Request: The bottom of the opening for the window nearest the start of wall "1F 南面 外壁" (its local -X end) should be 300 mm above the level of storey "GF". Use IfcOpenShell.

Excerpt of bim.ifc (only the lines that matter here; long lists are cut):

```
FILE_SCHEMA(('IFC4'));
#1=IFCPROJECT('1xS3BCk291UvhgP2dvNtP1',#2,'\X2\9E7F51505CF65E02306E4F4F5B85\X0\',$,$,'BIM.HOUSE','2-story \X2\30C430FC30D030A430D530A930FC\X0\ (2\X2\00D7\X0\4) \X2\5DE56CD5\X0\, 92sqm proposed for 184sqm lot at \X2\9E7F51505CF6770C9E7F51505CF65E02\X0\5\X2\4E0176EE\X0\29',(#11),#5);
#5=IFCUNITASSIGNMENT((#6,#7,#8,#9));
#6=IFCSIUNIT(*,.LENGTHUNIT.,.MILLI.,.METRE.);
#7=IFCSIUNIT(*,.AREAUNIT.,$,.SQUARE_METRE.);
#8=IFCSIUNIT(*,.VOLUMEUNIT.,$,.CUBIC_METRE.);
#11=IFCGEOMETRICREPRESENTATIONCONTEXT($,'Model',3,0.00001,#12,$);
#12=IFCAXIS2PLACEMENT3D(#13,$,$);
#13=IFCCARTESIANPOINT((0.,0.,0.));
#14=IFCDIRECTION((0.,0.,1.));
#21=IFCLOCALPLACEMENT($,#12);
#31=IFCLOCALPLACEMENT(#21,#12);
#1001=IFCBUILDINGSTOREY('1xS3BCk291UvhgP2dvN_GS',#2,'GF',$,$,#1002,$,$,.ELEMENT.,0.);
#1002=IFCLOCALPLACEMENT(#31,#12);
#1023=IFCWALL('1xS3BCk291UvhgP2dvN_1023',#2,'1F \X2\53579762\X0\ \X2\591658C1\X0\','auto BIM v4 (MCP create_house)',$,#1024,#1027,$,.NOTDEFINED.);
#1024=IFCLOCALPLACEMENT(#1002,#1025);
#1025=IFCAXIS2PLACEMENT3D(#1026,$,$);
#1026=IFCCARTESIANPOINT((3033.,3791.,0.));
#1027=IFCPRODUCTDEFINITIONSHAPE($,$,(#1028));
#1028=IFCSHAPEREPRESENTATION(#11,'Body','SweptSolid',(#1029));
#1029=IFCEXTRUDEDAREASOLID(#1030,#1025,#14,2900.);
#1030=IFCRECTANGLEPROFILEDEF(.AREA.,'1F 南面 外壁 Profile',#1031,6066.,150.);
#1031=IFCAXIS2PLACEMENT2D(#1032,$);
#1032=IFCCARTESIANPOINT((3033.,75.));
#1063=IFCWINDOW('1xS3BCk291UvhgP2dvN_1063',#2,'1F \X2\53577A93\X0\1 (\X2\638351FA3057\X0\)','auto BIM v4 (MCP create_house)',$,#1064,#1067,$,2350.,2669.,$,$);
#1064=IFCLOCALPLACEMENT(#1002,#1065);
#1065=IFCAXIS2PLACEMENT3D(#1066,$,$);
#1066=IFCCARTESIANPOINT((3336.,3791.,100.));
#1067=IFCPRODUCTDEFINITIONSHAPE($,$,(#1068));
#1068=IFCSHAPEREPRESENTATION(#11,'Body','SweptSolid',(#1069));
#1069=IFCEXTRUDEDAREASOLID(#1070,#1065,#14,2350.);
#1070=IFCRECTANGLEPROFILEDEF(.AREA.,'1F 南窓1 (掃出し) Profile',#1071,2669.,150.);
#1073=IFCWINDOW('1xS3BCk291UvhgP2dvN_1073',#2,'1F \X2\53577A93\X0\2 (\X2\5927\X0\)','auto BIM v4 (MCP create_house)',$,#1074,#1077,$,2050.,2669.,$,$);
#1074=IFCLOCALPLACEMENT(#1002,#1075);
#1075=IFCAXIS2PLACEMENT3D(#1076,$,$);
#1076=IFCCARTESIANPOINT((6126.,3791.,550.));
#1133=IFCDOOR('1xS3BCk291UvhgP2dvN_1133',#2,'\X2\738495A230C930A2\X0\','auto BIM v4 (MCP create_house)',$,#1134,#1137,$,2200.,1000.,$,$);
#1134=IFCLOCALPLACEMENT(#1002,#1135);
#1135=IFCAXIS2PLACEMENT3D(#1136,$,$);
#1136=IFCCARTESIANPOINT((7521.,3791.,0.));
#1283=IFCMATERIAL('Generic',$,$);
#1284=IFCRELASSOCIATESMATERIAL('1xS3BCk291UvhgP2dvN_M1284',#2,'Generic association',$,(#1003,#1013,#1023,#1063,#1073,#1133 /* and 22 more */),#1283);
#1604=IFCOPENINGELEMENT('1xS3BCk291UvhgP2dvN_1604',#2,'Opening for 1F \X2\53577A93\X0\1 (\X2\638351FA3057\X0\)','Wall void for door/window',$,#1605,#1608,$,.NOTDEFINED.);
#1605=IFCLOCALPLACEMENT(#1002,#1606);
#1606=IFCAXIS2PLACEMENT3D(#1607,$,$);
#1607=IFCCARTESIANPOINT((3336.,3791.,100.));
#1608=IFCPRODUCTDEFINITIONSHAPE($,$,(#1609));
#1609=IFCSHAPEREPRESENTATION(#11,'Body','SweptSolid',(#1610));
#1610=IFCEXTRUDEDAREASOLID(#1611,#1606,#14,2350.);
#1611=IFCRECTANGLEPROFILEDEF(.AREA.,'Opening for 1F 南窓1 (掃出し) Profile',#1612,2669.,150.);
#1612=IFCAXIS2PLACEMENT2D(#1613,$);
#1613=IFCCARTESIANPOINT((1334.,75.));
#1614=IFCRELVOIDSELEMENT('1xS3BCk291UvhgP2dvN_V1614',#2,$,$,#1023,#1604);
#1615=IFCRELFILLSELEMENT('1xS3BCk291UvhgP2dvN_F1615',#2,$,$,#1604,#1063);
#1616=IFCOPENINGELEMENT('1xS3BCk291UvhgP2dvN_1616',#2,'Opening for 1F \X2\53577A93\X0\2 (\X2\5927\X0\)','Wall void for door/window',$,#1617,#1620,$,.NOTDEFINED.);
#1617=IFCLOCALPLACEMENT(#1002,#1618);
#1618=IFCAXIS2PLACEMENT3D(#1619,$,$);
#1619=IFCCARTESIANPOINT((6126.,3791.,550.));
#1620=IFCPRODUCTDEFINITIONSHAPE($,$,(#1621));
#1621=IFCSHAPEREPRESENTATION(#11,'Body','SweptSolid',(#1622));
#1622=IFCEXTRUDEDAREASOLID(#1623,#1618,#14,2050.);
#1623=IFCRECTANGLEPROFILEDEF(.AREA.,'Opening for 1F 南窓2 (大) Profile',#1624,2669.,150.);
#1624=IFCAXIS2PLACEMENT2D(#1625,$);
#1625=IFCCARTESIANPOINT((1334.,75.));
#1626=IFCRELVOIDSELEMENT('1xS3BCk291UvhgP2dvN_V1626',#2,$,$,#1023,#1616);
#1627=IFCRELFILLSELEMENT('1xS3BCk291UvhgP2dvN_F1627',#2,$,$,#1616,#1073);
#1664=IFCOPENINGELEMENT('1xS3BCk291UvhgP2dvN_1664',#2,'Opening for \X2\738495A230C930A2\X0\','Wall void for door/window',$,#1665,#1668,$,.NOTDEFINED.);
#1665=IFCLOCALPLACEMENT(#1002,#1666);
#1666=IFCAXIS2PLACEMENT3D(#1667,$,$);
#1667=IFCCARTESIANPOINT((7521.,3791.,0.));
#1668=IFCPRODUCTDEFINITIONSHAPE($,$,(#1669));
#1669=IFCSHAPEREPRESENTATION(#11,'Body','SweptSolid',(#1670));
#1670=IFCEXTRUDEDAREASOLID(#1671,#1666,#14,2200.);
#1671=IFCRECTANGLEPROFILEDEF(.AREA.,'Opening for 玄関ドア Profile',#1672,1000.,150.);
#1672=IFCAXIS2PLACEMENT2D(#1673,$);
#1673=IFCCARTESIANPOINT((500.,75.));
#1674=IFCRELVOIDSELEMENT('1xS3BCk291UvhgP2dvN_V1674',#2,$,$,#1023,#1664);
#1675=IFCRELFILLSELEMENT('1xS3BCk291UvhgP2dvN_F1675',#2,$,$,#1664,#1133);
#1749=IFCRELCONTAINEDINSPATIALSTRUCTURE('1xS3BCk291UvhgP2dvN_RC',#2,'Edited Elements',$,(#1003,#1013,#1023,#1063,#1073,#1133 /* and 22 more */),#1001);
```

```python
import numpy as np
import ifcopenshell
import ifcopenshell.api.geometry
import ifcopenshell.geom
import ifcopenshell.util.element
import ifcopenshell.util.placement
import ifcopenshell.util.shape
import ifcopenshell.util.unit

model = ifcopenshell.open("bim.ifc")
unit_scale = ifcopenshell.util.unit.calculate_unit_scale(model)

window = model.by_id(1063)
opening = window.FillsVoids[0].RelatingOpeningElement
storey = ifcopenshell.util.element.get_container(window, ifc_class="IfcBuildingStorey")
level = ifcopenshell.util.placement.get_local_placement(storey.ObjectPlacement)[2, 3]

# The opening's origin need not be at the sill, so measure its lowest point.
shape = ifcopenshell.geom.create_shape(ifcopenshell.geom.settings(), opening)
bottom = ifcopenshell.util.shape.get_shape_bottom_elevation(shape, shape.geometry) / unit_scale
dz = level + 0.3 / unit_scale - bottom

shift = np.array([0.0, 0.0, dz])
# The window is not placed relative to its opening, so move both.
for product in (opening, window):
    matrix = ifcopenshell.util.placement.get_local_placement(product.ObjectPlacement)
    matrix[:3, 3] += shift
    ifcopenshell.api.geometry.edit_object_placement(model, product=product, matrix=matrix, is_si=False)

print(f"moved by {dz * unit_scale:+.3f} m")

model.write("bim_edited.ifc")
```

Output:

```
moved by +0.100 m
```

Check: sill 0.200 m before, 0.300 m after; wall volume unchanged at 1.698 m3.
